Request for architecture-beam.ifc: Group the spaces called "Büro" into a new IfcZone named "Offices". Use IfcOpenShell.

First a look at what the model holds.

```python
import ifcopenshell

model = ifcopenshell.open("architecture-beam.ifc")
print(model.schema)
seen = {}
for space in model.by_type("IfcSpace"):
    seen[space.LongName] = seen.get(space.LongName, 0) + 1
for name, count in sorted(seen.items(), key=str):
    print(count, "x", name)
print("zones:", [z.Name for z in model.by_type("IfcZone")][:20])
```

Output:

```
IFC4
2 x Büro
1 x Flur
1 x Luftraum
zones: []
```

```python
import ifcopenshell
import ifcopenshell.api.group
import ifcopenshell.api.root

model = ifcopenshell.open("architecture-beam.ifc")

names = {"Büro"}
spaces = [s for s in model.by_type("IfcSpace") if s.LongName in names]

zone = ifcopenshell.api.root.create_entity(model, ifc_class="IfcZone", name="Offices")
ifcopenshell.api.group.assign_group(model, products=spaces, group=zone)
print(len(spaces), "spaces in", zone.Name)

model.write("architecture-beam-out.ifc")
```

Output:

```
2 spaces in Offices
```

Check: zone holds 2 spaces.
